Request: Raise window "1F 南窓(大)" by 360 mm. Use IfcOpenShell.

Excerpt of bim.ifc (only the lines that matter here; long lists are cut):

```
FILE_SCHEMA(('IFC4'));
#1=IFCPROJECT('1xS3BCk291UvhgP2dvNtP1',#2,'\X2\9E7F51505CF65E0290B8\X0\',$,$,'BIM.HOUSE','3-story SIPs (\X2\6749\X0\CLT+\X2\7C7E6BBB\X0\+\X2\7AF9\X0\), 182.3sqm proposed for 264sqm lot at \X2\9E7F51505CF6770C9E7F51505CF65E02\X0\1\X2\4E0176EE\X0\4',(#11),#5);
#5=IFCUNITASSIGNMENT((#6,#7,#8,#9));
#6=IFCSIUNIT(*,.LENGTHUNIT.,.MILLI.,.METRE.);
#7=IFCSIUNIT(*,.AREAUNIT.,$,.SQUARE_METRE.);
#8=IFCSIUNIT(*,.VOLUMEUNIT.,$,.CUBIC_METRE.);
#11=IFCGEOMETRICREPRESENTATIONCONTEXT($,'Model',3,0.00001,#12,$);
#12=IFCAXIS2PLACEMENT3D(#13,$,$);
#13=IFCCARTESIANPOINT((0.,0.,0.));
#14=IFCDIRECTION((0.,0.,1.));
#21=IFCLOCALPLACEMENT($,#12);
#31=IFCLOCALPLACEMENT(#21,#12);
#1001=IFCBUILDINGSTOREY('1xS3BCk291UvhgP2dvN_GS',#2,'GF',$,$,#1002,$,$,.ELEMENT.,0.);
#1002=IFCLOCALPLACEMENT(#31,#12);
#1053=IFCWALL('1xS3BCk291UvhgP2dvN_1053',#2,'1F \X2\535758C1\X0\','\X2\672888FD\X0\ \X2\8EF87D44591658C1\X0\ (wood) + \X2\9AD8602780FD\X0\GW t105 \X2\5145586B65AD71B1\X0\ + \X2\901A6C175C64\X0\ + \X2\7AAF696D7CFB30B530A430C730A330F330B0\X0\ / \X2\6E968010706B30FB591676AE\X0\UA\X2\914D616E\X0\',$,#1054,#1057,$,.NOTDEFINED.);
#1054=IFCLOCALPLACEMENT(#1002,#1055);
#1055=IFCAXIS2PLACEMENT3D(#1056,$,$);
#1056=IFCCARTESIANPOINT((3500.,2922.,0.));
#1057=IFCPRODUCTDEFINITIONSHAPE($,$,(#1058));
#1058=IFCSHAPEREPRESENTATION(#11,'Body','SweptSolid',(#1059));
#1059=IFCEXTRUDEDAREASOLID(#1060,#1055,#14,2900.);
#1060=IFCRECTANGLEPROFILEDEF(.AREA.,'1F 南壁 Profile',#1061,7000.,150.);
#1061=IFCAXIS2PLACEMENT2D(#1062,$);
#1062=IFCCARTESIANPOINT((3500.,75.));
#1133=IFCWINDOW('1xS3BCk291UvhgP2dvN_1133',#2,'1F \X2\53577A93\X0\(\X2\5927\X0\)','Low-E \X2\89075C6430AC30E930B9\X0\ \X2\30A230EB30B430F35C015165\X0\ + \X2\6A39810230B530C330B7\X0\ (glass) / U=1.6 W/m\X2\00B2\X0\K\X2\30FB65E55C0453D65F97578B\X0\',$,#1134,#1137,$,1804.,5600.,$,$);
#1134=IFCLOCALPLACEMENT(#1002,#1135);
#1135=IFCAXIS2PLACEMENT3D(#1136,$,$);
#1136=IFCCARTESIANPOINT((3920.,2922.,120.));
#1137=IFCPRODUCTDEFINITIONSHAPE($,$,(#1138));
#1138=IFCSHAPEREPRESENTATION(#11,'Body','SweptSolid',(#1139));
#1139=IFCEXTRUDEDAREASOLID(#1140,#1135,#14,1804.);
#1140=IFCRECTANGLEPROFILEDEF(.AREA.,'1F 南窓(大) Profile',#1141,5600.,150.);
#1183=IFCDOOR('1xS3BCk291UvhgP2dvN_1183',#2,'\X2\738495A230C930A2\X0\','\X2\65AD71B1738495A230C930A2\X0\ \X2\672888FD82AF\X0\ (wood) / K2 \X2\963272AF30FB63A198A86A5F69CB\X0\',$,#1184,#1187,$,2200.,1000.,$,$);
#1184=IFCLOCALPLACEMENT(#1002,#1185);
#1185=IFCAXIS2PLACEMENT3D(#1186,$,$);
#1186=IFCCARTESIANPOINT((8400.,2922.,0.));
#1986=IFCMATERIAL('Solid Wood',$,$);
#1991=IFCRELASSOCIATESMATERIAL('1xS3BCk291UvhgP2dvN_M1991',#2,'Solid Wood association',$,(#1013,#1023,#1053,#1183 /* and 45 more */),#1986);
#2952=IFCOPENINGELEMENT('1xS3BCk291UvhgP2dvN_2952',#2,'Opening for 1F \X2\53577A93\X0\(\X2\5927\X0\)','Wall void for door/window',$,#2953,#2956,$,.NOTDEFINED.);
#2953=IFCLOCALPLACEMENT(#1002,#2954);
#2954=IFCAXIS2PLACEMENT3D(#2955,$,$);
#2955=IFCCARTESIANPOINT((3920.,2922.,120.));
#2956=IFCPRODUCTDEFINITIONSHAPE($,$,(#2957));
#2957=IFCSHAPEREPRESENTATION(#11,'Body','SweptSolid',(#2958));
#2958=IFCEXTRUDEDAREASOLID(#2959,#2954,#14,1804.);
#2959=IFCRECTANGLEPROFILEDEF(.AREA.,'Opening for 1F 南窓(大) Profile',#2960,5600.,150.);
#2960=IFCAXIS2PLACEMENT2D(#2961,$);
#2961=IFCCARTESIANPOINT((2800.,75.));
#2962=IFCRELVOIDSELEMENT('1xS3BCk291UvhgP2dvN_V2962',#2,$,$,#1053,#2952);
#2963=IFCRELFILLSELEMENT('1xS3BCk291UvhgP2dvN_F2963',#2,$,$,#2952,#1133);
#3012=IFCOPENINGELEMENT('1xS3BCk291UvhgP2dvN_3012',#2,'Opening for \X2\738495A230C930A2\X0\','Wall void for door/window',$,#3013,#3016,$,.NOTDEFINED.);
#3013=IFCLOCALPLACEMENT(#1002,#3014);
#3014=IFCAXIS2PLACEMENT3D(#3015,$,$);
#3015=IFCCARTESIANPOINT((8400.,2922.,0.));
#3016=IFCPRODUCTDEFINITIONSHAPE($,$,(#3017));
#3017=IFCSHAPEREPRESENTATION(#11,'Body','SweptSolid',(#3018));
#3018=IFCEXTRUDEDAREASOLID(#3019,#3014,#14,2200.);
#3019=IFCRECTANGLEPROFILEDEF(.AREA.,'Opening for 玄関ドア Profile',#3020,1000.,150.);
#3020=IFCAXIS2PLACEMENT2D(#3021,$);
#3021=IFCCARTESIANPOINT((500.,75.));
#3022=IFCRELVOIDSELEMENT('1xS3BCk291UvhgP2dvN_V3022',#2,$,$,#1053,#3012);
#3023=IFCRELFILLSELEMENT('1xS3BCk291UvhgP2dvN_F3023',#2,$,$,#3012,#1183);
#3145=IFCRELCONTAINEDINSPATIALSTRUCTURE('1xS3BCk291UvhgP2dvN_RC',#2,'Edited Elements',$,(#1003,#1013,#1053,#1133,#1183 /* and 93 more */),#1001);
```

```python
import numpy as np
import ifcopenshell
import ifcopenshell.api.geometry
import ifcopenshell.util.placement
import ifcopenshell.util.unit

model = ifcopenshell.open("bim.ifc")
unit_scale = ifcopenshell.util.unit.calculate_unit_scale(model)

window = model.by_guid("1xS3BCk291UvhgP2dvN_1133")
opening = window.FillsVoids[0].RelatingOpeningElement
dz = 360.0

shift = np.array([0.0, 0.0, dz])
# The window is not placed relative to its opening, so move both.
for product in (opening, window):
    matrix = ifcopenshell.util.placement.get_local_placement(product.ObjectPlacement)
    matrix[:3, 3] += shift
    ifcopenshell.api.geometry.edit_object_placement(model, product=product, matrix=matrix, is_si=False)

print(f"moved by {dz * unit_scale:+.3f} m")

model.write("bim-out.ifc")
```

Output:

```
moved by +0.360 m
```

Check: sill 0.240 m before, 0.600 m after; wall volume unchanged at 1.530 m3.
